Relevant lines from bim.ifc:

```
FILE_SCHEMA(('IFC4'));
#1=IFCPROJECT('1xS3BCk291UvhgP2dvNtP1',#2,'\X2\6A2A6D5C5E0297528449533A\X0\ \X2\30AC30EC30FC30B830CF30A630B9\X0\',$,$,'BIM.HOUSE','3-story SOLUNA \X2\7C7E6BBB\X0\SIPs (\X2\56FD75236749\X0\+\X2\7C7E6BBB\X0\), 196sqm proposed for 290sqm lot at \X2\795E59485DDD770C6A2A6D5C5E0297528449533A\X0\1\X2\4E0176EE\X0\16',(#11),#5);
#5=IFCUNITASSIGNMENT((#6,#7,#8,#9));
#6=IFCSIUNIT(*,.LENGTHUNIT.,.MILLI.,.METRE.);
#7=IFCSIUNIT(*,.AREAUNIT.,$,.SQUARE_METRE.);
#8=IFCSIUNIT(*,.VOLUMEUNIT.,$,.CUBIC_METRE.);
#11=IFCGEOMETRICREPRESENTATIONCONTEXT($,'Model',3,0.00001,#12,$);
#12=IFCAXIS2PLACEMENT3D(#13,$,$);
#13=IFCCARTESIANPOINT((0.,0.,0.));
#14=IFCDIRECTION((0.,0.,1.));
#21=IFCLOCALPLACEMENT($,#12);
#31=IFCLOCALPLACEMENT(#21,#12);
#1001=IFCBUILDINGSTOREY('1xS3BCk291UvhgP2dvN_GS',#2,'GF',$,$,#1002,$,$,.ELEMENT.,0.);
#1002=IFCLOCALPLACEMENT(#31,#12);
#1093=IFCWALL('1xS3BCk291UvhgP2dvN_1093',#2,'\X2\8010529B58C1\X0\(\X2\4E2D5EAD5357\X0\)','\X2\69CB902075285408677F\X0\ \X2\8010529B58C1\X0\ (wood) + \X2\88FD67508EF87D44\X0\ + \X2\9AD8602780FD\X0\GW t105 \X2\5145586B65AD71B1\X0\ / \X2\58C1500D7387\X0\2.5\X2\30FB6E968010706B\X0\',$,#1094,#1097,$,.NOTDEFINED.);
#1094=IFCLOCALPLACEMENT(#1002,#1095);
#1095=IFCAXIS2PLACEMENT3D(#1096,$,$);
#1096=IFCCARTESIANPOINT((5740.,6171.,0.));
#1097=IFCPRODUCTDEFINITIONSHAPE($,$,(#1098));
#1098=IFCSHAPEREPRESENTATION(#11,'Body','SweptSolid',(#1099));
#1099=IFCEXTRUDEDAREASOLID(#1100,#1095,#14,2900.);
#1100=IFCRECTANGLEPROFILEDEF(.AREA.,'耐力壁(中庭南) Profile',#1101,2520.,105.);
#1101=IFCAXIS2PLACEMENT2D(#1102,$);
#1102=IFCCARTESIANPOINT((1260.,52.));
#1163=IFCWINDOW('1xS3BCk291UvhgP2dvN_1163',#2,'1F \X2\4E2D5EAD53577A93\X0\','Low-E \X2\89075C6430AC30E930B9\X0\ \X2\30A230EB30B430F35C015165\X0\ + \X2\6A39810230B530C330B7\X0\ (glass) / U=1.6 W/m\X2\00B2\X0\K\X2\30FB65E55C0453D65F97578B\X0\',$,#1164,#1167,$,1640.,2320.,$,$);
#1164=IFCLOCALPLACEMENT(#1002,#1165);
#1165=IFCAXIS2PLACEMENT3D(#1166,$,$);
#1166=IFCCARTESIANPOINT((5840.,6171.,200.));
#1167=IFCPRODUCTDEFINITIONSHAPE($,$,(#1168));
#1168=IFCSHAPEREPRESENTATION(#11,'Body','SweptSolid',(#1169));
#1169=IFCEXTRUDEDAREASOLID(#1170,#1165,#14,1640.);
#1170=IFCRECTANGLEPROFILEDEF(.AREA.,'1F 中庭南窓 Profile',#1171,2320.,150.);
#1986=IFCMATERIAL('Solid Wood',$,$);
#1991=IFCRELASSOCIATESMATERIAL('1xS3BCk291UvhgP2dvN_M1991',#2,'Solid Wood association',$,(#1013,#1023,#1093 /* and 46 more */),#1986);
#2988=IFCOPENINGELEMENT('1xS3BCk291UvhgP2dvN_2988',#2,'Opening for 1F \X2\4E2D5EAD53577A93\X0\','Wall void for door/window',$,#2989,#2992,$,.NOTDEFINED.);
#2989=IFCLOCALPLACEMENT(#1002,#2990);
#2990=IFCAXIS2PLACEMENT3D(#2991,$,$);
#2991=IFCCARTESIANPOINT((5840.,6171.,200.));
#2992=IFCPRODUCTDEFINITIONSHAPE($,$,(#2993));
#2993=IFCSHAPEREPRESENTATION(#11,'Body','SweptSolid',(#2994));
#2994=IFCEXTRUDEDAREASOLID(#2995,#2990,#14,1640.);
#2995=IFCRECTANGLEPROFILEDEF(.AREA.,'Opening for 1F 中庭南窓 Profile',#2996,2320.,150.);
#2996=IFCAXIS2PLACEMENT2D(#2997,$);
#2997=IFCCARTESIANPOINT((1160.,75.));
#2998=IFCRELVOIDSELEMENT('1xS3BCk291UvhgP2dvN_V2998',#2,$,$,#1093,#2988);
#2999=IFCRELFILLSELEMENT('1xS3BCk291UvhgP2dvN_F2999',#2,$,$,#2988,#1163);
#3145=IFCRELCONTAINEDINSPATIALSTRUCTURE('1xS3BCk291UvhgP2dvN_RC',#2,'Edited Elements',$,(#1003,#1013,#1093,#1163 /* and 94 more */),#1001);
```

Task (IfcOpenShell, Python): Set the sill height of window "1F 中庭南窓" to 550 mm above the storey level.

```python
import numpy as np
import ifcopenshell
import ifcopenshell.api.geometry
import ifcopenshell.geom
import ifcopenshell.util.element
import ifcopenshell.util.placement
import ifcopenshell.util.shape
import ifcopenshell.util.unit

model = ifcopenshell.open("bim.ifc")
unit_scale = ifcopenshell.util.unit.calculate_unit_scale(model)

window = model.by_guid("1xS3BCk291UvhgP2dvN_1163")
opening = window.FillsVoids[0].RelatingOpeningElement
storey = ifcopenshell.util.element.get_container(window, ifc_class="IfcBuildingStorey")
level = ifcopenshell.util.placement.get_local_placement(storey.ObjectPlacement)[2, 3]

# The opening's origin need not be at the sill, so measure its lowest point.
shape = ifcopenshell.geom.create_shape(ifcopenshell.geom.settings(), opening)
bottom = ifcopenshell.util.shape.get_shape_bottom_elevation(shape, shape.geometry) / unit_scale
dz = level + 0.55 / unit_scale - bottom

shift = np.array([0.0, 0.0, dz])
# The window is not placed relative to its opening, so move both.
for product in (opening, window):
    matrix = ifcopenshell.util.placement.get_local_placement(product.ObjectPlacement)
    matrix[:3, 3] += shift
    ifcopenshell.api.geometry.edit_object_placement(model, product=product, matrix=matrix, is_si=False)

print(f"moved by {dz * unit_scale:+.3f} m")

model.write("bim_edited.ifc")
```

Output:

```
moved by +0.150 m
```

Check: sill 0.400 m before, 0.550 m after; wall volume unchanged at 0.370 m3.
